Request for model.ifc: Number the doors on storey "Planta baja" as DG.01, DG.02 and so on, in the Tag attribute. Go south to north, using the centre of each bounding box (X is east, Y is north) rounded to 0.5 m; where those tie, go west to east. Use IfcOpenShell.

First a look at what the model holds.

```python
import ifcopenshell
import ifcopenshell.util.element
import ifcopenshell.util.placement

model = ifcopenshell.open("model.ifc")
print(model.schema)
storey = next(s for s in model.by_type("IfcBuildingStorey") if s.Name == "Planta baja")
doors = [e for e in ifcopenshell.util.element.get_decomposition(storey) if e.is_a("IfcDoor")]
for e in sorted(doors, key=lambda e: e.id()):
    origin = ifcopenshell.util.placement.get_local_placement(e.ObjectPlacement)[:3, 3]
    print(e.id(), e.Tag, e.Name, origin.round(2) + 0.0, sep=" | ")
```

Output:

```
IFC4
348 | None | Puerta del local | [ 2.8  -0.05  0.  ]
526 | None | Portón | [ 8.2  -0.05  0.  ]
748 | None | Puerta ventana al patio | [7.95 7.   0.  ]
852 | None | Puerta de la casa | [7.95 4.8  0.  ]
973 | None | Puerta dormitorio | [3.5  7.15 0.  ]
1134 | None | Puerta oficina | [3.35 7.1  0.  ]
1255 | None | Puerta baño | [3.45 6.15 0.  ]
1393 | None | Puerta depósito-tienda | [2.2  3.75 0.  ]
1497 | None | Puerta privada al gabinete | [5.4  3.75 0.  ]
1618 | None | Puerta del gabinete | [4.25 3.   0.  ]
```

```python
import ifcopenshell
import ifcopenshell.geom
import ifcopenshell.util.element
import ifcopenshell.util.shape

model = ifcopenshell.open("model.ifc")
settings = ifcopenshell.geom.settings()
settings.set("use-world-coords", True)


def centre(element):
    shape = ifcopenshell.geom.create_shape(settings, element)
    return ifcopenshell.util.shape.get_bbox_centroid(shape.geometry)


storey = next(s for s in model.by_type("IfcBuildingStorey") if s.Name == "Planta baja")
doors = [e for e in ifcopenshell.util.element.get_decomposition(storey) if e.is_a("IfcDoor")]

# Insertion points can sit at a corner or the storey origin, so sort by the geometry (in metres).
centres = {e: centre(e) for e in doors}
doors.sort(key=lambda e: (round(centres[e][1] / 0.5), centres[e][0]))

for i, e in enumerate(doors, start=1):
    number = f"DG.{i:02d}"
    e.Tag = number
    print(e.id(), number)

model.write("model_updated.ifc")
```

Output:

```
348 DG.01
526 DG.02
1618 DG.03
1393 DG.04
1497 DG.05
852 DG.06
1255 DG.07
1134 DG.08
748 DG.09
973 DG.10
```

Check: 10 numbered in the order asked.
